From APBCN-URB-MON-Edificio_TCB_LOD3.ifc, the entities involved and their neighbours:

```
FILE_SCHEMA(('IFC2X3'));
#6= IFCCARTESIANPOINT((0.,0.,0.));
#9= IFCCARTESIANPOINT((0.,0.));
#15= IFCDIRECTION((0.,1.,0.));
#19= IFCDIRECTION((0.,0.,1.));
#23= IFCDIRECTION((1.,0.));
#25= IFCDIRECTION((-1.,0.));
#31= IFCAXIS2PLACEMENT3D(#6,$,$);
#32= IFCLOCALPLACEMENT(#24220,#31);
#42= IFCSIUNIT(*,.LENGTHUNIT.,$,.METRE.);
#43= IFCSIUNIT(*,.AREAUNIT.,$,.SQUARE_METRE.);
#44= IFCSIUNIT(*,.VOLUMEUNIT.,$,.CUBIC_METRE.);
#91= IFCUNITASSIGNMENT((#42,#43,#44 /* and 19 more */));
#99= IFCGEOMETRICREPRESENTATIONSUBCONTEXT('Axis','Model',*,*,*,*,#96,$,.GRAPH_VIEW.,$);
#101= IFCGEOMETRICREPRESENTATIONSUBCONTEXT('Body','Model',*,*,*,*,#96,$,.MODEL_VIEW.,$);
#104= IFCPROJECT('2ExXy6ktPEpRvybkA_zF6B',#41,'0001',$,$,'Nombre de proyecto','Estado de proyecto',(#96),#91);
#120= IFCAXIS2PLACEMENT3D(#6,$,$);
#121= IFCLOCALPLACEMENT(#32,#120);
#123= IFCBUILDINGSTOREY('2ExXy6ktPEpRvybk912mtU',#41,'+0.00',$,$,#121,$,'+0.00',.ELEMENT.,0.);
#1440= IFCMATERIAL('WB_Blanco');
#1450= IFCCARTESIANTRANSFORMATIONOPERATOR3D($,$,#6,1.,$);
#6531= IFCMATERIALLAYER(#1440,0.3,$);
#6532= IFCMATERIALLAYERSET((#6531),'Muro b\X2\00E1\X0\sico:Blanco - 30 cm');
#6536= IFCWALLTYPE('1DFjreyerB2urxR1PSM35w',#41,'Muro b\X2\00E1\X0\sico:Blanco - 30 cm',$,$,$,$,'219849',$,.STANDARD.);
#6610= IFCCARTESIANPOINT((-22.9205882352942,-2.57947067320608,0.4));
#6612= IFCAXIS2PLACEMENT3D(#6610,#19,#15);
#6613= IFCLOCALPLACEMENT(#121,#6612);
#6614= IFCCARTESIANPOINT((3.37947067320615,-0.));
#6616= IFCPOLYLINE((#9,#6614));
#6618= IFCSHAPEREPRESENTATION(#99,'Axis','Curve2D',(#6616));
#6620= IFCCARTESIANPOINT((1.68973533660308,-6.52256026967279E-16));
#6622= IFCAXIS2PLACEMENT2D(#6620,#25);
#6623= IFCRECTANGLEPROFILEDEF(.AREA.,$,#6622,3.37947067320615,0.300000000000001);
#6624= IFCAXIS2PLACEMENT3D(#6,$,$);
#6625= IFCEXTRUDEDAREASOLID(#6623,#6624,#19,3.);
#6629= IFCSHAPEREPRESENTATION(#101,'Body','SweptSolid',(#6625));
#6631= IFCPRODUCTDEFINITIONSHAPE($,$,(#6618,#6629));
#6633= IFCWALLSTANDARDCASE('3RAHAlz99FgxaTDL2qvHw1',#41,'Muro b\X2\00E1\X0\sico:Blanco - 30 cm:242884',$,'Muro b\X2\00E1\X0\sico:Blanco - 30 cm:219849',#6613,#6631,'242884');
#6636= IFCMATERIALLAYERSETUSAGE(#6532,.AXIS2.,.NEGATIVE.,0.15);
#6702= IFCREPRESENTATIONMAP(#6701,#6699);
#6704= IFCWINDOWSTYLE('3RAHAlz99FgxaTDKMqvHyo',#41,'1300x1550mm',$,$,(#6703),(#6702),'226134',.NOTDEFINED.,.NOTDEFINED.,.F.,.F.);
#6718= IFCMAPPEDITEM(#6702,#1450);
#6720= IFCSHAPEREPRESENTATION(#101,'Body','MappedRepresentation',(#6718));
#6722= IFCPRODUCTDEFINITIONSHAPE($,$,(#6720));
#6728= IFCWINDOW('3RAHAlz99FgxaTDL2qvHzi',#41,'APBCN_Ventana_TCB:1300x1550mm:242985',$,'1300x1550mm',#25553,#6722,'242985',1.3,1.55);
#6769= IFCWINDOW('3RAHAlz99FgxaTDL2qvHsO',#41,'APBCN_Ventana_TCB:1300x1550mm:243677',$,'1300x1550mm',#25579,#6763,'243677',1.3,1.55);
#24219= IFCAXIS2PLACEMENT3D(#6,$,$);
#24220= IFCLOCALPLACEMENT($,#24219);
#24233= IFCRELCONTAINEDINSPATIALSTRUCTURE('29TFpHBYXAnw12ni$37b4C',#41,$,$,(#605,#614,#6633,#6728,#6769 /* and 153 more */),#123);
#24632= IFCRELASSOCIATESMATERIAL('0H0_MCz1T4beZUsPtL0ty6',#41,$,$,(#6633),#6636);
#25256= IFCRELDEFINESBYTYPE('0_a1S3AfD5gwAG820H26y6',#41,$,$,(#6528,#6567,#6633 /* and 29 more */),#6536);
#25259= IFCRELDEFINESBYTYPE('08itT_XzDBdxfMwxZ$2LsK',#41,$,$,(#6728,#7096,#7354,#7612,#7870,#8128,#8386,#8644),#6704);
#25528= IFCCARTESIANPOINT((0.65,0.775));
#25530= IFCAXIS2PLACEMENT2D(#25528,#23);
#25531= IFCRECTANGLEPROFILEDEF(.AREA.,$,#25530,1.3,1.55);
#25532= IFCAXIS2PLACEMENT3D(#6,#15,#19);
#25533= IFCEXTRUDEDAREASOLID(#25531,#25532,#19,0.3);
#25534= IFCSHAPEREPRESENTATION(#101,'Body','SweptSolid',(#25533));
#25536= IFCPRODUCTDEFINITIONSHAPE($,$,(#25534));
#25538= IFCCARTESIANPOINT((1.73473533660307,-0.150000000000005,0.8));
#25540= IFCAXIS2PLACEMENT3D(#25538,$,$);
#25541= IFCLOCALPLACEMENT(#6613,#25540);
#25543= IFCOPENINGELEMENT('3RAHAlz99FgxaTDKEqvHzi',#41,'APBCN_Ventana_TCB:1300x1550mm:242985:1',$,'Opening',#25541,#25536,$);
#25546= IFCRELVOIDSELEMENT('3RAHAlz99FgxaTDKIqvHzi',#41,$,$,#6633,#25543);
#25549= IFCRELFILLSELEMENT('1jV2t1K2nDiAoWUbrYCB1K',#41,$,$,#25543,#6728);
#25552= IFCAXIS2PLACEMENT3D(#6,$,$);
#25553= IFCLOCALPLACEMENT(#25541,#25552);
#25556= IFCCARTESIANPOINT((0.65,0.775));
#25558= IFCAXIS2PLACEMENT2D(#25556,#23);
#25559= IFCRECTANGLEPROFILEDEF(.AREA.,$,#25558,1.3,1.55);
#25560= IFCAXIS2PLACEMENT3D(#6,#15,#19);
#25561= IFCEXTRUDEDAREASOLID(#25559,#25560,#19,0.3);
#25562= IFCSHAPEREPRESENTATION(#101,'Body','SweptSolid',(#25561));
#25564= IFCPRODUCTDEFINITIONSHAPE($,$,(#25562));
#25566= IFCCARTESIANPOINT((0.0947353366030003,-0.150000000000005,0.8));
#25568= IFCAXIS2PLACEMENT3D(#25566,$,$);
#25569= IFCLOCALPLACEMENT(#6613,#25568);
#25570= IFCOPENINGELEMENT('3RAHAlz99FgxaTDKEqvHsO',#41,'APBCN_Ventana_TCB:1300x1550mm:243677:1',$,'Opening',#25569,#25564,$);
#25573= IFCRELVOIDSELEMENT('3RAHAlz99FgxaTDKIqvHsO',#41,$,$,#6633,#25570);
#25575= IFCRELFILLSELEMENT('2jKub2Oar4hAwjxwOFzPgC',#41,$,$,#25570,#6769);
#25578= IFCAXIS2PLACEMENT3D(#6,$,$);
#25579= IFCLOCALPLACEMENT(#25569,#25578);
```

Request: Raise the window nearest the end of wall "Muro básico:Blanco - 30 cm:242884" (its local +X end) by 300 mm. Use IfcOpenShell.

```python
import numpy as np
import ifcopenshell
import ifcopenshell.api.geometry
import ifcopenshell.util.placement
import ifcopenshell.util.unit

model = ifcopenshell.open("APBCN-URB-MON-Edificio_TCB_LOD3.ifc")
unit_scale = ifcopenshell.util.unit.calculate_unit_scale(model)

window = model.by_guid("3RAHAlz99FgxaTDL2qvHzi")
opening = window.FillsVoids[0].RelatingOpeningElement
dz = 0.3 / unit_scale

shift = np.array([0.0, 0.0, dz])
# The window is placed relative to its opening, so it follows when the opening moves.
matrix = ifcopenshell.util.placement.get_local_placement(opening.ObjectPlacement)
matrix[:3, 3] += shift
ifcopenshell.api.geometry.edit_object_placement(
    model, product=opening, matrix=matrix, is_si=False, should_transform_children=True
)

print(f"moved by {dz * unit_scale:+.3f} m")

model.write("APBCN-URB-MON-Edificio_TCB_LOD3_updated.ifc")
```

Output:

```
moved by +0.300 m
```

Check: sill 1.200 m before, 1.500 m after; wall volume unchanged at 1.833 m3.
